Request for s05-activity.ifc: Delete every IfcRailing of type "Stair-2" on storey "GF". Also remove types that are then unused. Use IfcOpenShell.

First a look at what the model holds.

```python
import ifcopenshell
import ifcopenshell.util.element

model = ifcopenshell.open("s05-activity.ifc")
print(model.schema)
storey = next(s for s in model.by_type("IfcBuildingStorey") if s.Name == "GF")
railings = [e for e in ifcopenshell.util.element.get_decomposition(storey) if e.is_a("IfcRailing")]
seen = {}
for e in railings:
    element_type = ifcopenshell.util.element.get_type(e)
    name = element_type.Name if element_type not in (None, e) else None
    seen[name] = seen.get(name, 0) + 1
for name, count in sorted(seen.items(), key=str):
    print(count, "x", name)
```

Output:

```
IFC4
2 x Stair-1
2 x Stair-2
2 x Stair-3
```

```python
import ifcopenshell
import ifcopenshell.api.root
import ifcopenshell.util.element

model = ifcopenshell.open("s05-activity.ifc")

storey = next(s for s in model.by_type("IfcBuildingStorey") if s.Name == "GF")
railings = [e for e in ifcopenshell.util.element.get_decomposition(storey) if e.is_a("IfcRailing")]
targets = [e for e in railings if (t := ifcopenshell.util.element.get_type(e)) not in (None, e) and t.Name == "Stair-2"]
types = {ifcopenshell.util.element.get_type(e) for e in targets} - {None, *targets}

for e in targets:
    ifcopenshell.api.root.remove_product(model, product=e)
print(len(targets), "removed")

unused = [t for t in types if not ifcopenshell.util.element.get_types(t)]
for t in unused:
    ifcopenshell.api.root.remove_product(model, product=t)
print(len(unused), "unused types removed")

model.write("s05-activity-out.ifc")
```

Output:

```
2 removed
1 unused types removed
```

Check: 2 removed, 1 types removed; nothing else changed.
